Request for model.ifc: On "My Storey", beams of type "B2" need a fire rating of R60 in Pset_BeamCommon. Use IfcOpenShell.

First a look at what the model holds.

```python
import ifcopenshell
import ifcopenshell.util.element

model = ifcopenshell.open("model.ifc")
print(model.schema)
storey = next(s for s in model.by_type("IfcBuildingStorey") if s.Name == "My Storey")
beams = [e for e in ifcopenshell.util.element.get_decomposition(storey) if e.is_a("IfcBeam")]
seen = {}
for e in beams:
    element_type = ifcopenshell.util.element.get_type(e)
    key = (element_type.Name if element_type != e and element_type else None, ifcopenshell.util.element.get_pset(e, "Pset_BeamCommon", "FireRating"))
    seen[key] = seen.get(key, 0) + 1
for (name, value), count in sorted(seen.items(), key=str):
    print(count, "x", name, "|", value)
```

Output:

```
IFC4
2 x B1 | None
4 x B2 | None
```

```python
import ifcopenshell
import ifcopenshell.api.pset
import ifcopenshell.util.element

model = ifcopenshell.open("model.ifc")

storey = next(s for s in model.by_type("IfcBuildingStorey") if s.Name == "My Storey")
beams = [e for e in ifcopenshell.util.element.get_decomposition(storey) if e.is_a("IfcBeam")]

count = 0
for e in beams:
    element_type = ifcopenshell.util.element.get_type(e)
    if element_type in (None, e) or element_type.Name != "B2":
        continue
    # add_pset returns the element's existing set when there is one.
    pset = ifcopenshell.api.pset.add_pset(model, product=e, name="Pset_BeamCommon")
    ifcopenshell.api.pset.edit_pset(model, pset=pset, properties={"FireRating": "R60"})
    count += 1

print(count, "beams updated")

model.write("model_updated.ifc")
```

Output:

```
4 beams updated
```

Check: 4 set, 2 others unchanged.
